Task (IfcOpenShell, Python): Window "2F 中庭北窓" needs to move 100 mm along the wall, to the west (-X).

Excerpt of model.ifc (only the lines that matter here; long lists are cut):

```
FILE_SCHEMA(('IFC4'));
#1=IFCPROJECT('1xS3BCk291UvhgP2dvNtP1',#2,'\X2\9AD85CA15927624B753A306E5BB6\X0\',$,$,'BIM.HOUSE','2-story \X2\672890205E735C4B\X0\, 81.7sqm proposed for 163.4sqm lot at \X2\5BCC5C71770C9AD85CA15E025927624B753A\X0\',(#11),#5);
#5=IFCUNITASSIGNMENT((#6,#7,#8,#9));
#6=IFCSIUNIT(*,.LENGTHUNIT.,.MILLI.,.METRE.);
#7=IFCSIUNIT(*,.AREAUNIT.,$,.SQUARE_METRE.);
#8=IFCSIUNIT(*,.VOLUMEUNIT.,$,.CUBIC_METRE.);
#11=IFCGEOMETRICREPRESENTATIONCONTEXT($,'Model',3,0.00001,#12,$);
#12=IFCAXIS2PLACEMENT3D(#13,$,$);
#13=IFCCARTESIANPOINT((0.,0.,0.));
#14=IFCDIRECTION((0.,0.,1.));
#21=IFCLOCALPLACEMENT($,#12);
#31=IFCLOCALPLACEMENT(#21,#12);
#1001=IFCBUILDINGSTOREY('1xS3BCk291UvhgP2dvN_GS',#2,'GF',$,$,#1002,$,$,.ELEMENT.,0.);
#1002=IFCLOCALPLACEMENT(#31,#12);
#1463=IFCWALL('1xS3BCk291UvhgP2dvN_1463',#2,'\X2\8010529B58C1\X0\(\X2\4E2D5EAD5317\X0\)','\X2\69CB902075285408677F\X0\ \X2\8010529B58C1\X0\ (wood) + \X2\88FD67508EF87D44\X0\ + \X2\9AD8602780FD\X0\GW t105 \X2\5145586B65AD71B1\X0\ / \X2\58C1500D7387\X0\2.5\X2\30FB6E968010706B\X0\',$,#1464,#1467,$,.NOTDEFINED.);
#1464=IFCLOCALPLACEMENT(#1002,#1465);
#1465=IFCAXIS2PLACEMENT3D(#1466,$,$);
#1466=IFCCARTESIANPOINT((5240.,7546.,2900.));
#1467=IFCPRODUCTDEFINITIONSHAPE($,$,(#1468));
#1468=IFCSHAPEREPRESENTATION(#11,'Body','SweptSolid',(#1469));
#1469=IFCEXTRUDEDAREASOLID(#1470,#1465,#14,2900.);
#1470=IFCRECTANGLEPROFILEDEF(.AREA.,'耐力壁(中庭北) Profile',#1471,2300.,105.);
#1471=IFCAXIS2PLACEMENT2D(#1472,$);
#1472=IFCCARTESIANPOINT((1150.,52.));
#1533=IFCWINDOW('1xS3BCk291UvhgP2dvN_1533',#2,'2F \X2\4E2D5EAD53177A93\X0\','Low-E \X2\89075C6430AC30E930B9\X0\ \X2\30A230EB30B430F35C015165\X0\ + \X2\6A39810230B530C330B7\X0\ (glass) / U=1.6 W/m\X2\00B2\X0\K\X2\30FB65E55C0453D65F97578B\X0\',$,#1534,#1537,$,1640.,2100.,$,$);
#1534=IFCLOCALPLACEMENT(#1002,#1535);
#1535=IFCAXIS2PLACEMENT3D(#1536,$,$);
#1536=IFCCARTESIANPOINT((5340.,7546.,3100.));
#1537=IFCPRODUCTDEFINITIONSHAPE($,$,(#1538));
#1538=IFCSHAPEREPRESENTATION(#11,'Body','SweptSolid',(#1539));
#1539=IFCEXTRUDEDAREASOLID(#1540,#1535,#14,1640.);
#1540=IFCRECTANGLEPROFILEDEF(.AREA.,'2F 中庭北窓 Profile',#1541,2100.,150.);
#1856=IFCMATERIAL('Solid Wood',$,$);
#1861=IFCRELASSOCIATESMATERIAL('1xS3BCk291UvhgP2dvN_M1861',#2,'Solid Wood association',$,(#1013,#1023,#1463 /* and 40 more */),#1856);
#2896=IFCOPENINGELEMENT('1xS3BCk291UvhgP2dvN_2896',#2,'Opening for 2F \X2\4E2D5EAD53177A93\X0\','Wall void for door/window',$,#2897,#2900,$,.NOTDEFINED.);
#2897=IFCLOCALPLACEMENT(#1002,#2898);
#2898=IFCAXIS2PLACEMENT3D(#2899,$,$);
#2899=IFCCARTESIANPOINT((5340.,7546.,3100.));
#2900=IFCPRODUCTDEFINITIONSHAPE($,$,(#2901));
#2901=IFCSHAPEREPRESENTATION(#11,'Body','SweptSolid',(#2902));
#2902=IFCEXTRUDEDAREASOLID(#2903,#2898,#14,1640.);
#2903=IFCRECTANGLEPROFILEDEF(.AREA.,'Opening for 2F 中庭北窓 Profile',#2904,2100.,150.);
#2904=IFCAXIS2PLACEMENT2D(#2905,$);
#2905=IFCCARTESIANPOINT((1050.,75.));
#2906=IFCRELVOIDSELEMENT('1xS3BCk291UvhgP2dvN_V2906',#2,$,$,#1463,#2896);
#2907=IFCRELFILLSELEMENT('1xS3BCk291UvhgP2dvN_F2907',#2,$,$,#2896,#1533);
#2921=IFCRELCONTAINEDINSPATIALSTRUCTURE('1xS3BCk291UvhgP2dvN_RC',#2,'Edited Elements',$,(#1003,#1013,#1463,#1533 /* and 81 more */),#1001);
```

```python
import ifcopenshell
import ifcopenshell.api.geometry
import ifcopenshell.util.placement

model = ifcopenshell.open("model.ifc")

window = model.by_guid("1xS3BCk291UvhgP2dvN_1533")
opening = window.FillsVoids[0].RelatingOpeningElement
wall = opening.VoidsElements[0].RelatingBuildingElement

wall_matrix = ifcopenshell.util.placement.get_local_placement(wall.ObjectPlacement)
shift = wall_matrix[:3, 0] * -100.0
before = ifcopenshell.util.placement.get_local_placement(window.ObjectPlacement)[:3, 3].copy()

# The window is not placed relative to its opening, so move both.
for product in (opening, window):
    matrix = ifcopenshell.util.placement.get_local_placement(product.ObjectPlacement)
    matrix[:3, 3] += shift
    ifcopenshell.api.geometry.edit_object_placement(model, product=product, matrix=matrix, is_si=False)

after = ifcopenshell.util.placement.get_local_placement(window.ObjectPlacement)[:3, 3]
print("window moved by", (after - before).round(3) + 0.0)

model.write("model_v2.ifc")
```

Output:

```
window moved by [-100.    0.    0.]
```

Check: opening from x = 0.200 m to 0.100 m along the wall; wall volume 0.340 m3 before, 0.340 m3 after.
